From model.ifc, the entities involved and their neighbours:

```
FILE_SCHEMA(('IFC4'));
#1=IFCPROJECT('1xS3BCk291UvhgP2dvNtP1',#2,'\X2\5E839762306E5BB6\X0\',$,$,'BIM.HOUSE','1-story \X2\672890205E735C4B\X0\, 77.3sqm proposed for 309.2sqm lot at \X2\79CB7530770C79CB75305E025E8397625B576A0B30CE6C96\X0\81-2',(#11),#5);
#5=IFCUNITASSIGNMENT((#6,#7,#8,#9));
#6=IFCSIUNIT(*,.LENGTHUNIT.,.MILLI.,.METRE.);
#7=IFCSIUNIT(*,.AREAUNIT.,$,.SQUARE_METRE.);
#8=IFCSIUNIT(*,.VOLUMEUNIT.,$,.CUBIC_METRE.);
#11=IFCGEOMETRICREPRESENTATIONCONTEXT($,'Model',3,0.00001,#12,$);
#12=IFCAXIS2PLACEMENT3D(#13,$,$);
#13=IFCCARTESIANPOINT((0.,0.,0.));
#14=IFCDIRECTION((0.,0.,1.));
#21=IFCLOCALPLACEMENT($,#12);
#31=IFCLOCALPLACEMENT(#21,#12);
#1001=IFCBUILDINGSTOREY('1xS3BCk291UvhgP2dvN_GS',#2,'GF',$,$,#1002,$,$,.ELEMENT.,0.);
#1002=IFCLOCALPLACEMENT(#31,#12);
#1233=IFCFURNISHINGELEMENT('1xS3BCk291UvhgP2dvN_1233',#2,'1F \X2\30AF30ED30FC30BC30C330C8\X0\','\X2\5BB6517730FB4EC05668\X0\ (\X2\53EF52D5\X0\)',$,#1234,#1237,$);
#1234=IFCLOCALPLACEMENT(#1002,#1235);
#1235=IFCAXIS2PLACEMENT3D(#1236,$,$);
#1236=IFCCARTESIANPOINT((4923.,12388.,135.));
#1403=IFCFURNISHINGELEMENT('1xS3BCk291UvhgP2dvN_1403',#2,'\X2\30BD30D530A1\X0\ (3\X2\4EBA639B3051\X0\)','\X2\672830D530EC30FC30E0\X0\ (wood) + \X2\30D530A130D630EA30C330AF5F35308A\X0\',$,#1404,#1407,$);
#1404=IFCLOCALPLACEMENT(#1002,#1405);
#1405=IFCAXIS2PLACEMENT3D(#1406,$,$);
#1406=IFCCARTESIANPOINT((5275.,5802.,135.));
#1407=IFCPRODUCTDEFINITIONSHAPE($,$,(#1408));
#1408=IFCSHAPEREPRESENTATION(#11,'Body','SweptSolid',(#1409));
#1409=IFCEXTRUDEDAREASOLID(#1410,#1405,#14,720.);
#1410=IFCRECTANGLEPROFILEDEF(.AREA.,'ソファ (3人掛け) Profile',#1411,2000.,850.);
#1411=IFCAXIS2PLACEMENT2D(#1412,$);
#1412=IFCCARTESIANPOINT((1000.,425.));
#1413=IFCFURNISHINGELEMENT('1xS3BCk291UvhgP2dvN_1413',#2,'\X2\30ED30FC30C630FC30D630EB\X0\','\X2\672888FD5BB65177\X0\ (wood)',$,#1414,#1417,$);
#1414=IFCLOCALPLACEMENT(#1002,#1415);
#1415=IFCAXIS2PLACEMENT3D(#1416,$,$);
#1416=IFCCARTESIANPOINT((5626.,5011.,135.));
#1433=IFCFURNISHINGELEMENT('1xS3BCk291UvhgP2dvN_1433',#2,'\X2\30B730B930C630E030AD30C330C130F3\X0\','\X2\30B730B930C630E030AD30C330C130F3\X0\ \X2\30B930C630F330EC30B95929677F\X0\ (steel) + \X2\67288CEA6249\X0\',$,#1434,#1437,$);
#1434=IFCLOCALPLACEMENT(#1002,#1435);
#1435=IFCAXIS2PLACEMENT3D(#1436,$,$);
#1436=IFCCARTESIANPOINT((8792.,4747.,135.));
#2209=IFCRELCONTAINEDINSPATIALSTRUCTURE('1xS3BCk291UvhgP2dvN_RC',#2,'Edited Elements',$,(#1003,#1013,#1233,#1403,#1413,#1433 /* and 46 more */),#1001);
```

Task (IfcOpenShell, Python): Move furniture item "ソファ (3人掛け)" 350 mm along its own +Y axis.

```python
import ifcopenshell
import ifcopenshell.api.geometry
import ifcopenshell.util.placement
import ifcopenshell.util.unit

model = ifcopenshell.open("model.ifc")
unit_scale = ifcopenshell.util.unit.calculate_unit_scale(model)

item = model.by_id(1403)
matrix = ifcopenshell.util.placement.get_local_placement(item.ObjectPlacement)
matrix[:3, 3] += matrix[:3, 1] * 0.35 / unit_scale
ifcopenshell.api.geometry.edit_object_placement(model, product=item, matrix=matrix, is_si=False)

print(ifcopenshell.util.placement.get_local_placement(item.ObjectPlacement).round(3) + 0.0)

model.write("model_rev.ifc")
```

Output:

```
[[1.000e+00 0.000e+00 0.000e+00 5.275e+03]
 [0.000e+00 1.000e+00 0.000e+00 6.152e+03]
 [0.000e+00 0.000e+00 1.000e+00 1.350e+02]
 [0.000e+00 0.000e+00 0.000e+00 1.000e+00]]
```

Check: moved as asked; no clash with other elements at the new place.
